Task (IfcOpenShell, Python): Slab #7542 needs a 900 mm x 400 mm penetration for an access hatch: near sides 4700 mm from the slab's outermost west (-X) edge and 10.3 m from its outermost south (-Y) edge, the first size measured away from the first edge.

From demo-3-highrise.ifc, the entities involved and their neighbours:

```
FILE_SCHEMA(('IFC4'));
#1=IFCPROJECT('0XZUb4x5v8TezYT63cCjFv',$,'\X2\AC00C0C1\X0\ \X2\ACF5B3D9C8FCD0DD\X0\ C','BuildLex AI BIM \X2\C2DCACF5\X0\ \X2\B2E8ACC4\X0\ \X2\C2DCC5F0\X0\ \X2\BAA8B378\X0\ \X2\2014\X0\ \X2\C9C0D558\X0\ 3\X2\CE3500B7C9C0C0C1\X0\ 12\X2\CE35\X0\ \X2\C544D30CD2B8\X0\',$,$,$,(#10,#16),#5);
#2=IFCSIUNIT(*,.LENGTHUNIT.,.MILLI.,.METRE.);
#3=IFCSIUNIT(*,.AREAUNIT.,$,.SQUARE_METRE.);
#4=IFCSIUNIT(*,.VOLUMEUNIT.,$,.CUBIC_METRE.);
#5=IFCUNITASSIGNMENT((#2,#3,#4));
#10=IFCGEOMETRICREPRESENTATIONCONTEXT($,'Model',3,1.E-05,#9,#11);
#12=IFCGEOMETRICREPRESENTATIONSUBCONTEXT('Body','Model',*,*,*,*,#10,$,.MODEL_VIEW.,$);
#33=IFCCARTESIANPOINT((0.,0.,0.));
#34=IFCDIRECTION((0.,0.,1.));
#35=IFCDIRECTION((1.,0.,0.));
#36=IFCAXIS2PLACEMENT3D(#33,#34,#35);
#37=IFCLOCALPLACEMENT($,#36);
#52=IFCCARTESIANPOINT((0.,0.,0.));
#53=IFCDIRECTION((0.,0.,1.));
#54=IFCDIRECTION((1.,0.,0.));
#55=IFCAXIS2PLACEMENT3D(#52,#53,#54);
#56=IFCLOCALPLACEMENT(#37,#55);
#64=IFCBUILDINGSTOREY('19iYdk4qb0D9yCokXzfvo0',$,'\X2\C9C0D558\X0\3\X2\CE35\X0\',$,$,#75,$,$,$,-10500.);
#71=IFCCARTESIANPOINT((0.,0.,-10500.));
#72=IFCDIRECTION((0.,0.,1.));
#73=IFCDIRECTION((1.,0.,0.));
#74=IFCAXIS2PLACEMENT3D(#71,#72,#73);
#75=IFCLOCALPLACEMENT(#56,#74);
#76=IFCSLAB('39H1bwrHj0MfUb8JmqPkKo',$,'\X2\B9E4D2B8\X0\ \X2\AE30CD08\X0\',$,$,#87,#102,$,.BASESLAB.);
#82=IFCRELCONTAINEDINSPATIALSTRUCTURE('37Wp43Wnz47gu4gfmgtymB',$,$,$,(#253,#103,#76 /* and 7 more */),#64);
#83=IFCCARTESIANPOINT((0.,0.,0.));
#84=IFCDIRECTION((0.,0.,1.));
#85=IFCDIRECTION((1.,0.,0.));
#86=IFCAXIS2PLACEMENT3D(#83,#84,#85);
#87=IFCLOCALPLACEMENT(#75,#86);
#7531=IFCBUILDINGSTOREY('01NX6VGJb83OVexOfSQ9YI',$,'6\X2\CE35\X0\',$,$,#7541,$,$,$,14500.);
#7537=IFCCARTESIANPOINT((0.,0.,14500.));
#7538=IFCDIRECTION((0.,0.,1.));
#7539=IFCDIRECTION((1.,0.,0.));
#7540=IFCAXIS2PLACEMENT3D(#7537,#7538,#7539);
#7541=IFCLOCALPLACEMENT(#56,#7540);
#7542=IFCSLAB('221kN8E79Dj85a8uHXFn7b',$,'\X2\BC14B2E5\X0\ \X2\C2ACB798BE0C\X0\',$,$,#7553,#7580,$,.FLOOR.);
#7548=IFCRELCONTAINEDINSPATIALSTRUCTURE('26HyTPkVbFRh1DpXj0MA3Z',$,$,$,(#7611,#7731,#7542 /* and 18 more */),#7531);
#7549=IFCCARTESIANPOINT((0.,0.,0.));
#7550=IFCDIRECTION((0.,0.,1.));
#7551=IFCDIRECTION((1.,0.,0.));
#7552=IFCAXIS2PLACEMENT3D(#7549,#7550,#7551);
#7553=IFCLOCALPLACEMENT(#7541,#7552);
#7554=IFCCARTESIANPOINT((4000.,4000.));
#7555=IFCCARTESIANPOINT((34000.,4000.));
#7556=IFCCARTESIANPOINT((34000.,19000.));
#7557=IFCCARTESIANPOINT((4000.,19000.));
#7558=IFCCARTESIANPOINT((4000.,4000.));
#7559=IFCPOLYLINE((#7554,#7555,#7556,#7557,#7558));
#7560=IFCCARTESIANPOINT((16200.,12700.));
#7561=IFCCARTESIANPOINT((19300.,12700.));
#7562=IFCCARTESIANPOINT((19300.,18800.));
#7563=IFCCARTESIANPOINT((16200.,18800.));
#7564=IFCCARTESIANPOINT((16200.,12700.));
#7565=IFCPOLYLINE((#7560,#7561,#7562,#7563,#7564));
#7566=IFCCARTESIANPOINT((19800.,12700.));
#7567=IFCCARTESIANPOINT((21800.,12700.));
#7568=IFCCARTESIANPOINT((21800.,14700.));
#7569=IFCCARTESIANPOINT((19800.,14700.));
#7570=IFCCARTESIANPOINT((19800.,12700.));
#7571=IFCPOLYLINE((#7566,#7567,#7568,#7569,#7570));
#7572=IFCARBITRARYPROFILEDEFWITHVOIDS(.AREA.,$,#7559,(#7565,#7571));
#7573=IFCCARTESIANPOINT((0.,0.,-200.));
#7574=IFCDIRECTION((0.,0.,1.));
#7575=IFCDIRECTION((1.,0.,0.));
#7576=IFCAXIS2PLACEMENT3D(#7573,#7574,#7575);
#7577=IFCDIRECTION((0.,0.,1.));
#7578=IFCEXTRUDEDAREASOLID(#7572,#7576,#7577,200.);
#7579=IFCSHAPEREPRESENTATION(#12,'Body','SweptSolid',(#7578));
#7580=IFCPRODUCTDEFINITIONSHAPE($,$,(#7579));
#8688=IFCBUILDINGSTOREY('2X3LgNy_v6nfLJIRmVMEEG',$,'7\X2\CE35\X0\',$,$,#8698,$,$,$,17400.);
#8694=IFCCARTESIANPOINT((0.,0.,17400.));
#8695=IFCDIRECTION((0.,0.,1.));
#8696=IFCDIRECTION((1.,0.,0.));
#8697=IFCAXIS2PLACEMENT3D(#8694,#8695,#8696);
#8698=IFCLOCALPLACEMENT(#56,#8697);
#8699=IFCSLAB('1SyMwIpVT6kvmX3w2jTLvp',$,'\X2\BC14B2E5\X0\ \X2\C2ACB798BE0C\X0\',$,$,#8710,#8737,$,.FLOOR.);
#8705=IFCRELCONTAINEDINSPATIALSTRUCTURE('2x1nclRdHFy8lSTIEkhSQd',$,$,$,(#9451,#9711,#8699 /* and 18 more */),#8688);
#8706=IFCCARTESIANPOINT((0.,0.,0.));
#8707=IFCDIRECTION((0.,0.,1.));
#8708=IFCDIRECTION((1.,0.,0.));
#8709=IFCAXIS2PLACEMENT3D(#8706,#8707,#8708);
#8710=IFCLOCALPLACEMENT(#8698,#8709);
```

```python
import numpy as np
import ifcopenshell
import ifcopenshell.api.feature
import ifcopenshell.api.geometry
import ifcopenshell.api.root
import ifcopenshell.geom
import ifcopenshell.util.placement
import ifcopenshell.util.representation
import ifcopenshell.util.shape
import ifcopenshell.util.unit

model = ifcopenshell.open("demo-3-highrise.ifc")
unit_scale = ifcopenshell.util.unit.calculate_unit_scale(model)
settings = ifcopenshell.geom.settings()


def volume(element):
    """Net volume in cubic metres, openings subtracted."""
    shape = ifcopenshell.geom.create_shape(settings, element)
    return ifcopenshell.util.shape.get_volume(shape.geometry)


slab = model.by_id(7542)
before = volume(slab)

# Extent in the slab's own axes, in metres. The edges named are its -X and -Y sides.
slab_shape = ifcopenshell.geom.create_shape(settings, slab)
vertices = ifcopenshell.util.shape.get_vertices(slab_shape.geometry)
x_min, y_min, bottom = vertices.min(axis=0)
top = vertices[:, 2].max()

opening = ifcopenshell.api.root.create_entity(model, ifc_class="IfcOpeningElement", name="Access hatch opening", predefined_type="OPENING")
context = ifcopenshell.util.representation.get_context(model, "Model", "Body", "MODEL_VIEW")
width, depth = 0.9, 0.4
outline = [(0.0, 0.0), (width, 0.0), (width, depth), (0.0, depth), (0.0, 0.0)]
# Overshoot both faces by 50 mm so the cut is clean.
shape = ifcopenshell.api.geometry.add_slab_representation(
    model, context=context, depth=top - bottom + 0.1, polyline=outline
)
ifcopenshell.api.geometry.assign_representation(model, product=opening, representation=shape)

matrix = ifcopenshell.util.placement.get_local_placement(slab.ObjectPlacement)
matrix[:, 3] = matrix @ np.append(np.array([x_min + 4.7, y_min + 10.3, bottom - 0.05]) / unit_scale, 1.0)
ifcopenshell.api.geometry.edit_object_placement(model, product=opening, matrix=matrix, is_si=False)
ifcopenshell.api.feature.add_feature(model, feature=opening, element=slab)

after = volume(slab)

print(f"slab volume {before:.3f} -> {after:.3f} m3")

model.write("demo-3-highrise_v2.ifc")
```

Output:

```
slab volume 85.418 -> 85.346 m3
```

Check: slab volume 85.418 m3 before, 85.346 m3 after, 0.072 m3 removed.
